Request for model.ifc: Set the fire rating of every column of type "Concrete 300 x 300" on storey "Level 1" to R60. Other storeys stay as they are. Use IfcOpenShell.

First a look at what the model holds.

```python
import ifcopenshell
import ifcopenshell.util.element

model = ifcopenshell.open("model.ifc")
print(model.schema)
storey = next(s for s in model.by_type("IfcBuildingStorey") if s.Name == "Level 1")
columns = [e for e in ifcopenshell.util.element.get_decomposition(storey) if e.is_a("IfcColumn")]
seen = {}
for e in columns:
    element_type = ifcopenshell.util.element.get_type(e)
    key = (element_type.Name if element_type != e and element_type else None, ifcopenshell.util.element.get_pset(e, "Pset_ColumnCommon", "FireRating"))
    seen[key] = seen.get(key, 0) + 1
for (name, value), count in sorted(seen.items(), key=str):
    print(count, "x", name, "|", value)
```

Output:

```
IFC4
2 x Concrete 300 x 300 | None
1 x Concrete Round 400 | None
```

```python
import ifcopenshell
import ifcopenshell.api.pset
import ifcopenshell.util.element

model = ifcopenshell.open("model.ifc")

storey = next(s for s in model.by_type("IfcBuildingStorey") if s.Name == "Level 1")
columns = [e for e in ifcopenshell.util.element.get_decomposition(storey) if e.is_a("IfcColumn")]

count = 0
for e in columns:
    element_type = ifcopenshell.util.element.get_type(e)
    if element_type in (None, e) or element_type.Name != "Concrete 300 x 300":
        continue
    # add_pset returns the element's existing set when there is one.
    pset = ifcopenshell.api.pset.add_pset(model, product=e, name="Pset_ColumnCommon")
    ifcopenshell.api.pset.edit_pset(model, pset=pset, properties={"FireRating": "R60"})
    count += 1

print(count, "columns updated")

model.write("model-out.ifc")
```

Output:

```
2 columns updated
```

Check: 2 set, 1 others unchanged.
